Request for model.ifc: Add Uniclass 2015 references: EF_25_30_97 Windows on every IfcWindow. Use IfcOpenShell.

First a look at what the model holds.

```python
import ifcopenshell

model = ifcopenshell.open("model.ifc")
print(model.schema)
print("classifications:", [c.Name for c in model.by_type("IfcClassification")])
for ifc_class in ("IfcDoor", "IfcRoof", "IfcStair", "IfcWall", "IfcWindow"):
    print(ifc_class, len(model.by_type(ifc_class)))
```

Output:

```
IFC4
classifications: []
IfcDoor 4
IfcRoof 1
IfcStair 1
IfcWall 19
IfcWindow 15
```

```python
import ifcopenshell
import ifcopenshell.api.classification

model = ifcopenshell.open("model.ifc")

system = ifcopenshell.api.classification.add_classification(model, classification="Uniclass 2015")

codes = {
    "IfcWindow": ("EF_25_30_97", "Windows"),
}
for ifc_class, (code, name) in codes.items():
    products = model.by_type(ifc_class)
    ifcopenshell.api.classification.add_reference(
        model, products=products, classification=system, identification=code, name=name
    )
    print(code, len(products))

model.write("model-out.ifc")
```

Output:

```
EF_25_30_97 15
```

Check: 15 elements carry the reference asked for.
